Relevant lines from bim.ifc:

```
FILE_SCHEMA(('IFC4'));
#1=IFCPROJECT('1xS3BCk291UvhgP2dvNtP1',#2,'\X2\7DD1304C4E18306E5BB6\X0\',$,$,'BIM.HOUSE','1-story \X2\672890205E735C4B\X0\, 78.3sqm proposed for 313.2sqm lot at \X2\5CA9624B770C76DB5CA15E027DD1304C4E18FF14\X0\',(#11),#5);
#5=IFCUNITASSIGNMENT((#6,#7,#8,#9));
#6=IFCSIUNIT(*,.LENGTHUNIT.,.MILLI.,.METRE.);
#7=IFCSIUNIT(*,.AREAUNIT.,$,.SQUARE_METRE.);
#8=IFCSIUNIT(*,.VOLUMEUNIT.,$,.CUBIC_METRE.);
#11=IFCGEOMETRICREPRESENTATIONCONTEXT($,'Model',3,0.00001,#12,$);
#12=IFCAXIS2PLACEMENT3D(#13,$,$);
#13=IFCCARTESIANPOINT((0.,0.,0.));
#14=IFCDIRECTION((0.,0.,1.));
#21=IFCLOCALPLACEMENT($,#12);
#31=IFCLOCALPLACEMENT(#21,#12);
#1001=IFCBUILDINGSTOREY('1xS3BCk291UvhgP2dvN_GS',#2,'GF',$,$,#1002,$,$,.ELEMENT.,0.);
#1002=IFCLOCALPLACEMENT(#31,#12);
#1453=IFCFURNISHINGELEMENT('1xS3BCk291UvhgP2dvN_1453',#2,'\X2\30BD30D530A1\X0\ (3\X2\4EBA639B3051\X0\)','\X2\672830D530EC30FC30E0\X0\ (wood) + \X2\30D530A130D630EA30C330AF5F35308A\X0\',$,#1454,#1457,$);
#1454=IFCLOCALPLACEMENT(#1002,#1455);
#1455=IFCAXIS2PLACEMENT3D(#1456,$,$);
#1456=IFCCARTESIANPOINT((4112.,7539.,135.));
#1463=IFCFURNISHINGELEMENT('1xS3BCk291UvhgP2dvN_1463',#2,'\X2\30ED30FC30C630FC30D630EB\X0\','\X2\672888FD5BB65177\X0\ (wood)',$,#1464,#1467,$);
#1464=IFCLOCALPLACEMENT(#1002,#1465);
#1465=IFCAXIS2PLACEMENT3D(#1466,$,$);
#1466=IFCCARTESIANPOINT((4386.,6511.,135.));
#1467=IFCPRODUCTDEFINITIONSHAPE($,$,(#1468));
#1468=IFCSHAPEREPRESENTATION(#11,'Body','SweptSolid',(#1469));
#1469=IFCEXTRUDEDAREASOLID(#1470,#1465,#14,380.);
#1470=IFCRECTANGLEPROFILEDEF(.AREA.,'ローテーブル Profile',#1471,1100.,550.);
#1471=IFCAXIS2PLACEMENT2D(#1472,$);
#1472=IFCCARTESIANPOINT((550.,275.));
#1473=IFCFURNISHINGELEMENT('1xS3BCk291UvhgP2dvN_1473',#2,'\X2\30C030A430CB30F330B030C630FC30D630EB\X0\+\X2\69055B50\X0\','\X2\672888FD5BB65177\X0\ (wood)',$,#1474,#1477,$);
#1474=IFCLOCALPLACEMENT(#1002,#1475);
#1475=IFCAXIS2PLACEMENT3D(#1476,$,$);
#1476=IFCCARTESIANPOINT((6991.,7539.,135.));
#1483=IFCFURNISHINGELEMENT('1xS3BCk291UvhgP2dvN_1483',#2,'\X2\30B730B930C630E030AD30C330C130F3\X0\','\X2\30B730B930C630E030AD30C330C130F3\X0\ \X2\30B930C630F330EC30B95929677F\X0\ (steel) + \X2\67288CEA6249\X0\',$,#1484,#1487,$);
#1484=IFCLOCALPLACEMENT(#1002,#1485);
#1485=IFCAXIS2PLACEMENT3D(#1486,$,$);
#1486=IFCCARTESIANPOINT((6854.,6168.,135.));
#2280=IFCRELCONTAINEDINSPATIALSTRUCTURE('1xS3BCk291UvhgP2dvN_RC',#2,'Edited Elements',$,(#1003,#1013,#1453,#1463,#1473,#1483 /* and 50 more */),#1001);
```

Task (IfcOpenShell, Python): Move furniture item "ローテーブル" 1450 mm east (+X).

```python
import ifcopenshell
import ifcopenshell.api.geometry
import ifcopenshell.util.placement
import ifcopenshell.util.unit

model = ifcopenshell.open("bim.ifc")
unit_scale = ifcopenshell.util.unit.calculate_unit_scale(model)

item = model.by_guid("1xS3BCk291UvhgP2dvN_1463")
matrix = ifcopenshell.util.placement.get_local_placement(item.ObjectPlacement)
matrix[0, 3] += 1.45 / unit_scale
ifcopenshell.api.geometry.edit_object_placement(model, product=item, matrix=matrix, is_si=False)

print(ifcopenshell.util.placement.get_local_placement(item.ObjectPlacement).round(3) + 0.0)

model.write("bim-out.ifc")
```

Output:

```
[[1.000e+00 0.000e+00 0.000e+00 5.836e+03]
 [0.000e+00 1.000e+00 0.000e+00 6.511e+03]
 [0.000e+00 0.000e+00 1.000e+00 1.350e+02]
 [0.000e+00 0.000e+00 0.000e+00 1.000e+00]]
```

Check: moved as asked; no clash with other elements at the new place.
